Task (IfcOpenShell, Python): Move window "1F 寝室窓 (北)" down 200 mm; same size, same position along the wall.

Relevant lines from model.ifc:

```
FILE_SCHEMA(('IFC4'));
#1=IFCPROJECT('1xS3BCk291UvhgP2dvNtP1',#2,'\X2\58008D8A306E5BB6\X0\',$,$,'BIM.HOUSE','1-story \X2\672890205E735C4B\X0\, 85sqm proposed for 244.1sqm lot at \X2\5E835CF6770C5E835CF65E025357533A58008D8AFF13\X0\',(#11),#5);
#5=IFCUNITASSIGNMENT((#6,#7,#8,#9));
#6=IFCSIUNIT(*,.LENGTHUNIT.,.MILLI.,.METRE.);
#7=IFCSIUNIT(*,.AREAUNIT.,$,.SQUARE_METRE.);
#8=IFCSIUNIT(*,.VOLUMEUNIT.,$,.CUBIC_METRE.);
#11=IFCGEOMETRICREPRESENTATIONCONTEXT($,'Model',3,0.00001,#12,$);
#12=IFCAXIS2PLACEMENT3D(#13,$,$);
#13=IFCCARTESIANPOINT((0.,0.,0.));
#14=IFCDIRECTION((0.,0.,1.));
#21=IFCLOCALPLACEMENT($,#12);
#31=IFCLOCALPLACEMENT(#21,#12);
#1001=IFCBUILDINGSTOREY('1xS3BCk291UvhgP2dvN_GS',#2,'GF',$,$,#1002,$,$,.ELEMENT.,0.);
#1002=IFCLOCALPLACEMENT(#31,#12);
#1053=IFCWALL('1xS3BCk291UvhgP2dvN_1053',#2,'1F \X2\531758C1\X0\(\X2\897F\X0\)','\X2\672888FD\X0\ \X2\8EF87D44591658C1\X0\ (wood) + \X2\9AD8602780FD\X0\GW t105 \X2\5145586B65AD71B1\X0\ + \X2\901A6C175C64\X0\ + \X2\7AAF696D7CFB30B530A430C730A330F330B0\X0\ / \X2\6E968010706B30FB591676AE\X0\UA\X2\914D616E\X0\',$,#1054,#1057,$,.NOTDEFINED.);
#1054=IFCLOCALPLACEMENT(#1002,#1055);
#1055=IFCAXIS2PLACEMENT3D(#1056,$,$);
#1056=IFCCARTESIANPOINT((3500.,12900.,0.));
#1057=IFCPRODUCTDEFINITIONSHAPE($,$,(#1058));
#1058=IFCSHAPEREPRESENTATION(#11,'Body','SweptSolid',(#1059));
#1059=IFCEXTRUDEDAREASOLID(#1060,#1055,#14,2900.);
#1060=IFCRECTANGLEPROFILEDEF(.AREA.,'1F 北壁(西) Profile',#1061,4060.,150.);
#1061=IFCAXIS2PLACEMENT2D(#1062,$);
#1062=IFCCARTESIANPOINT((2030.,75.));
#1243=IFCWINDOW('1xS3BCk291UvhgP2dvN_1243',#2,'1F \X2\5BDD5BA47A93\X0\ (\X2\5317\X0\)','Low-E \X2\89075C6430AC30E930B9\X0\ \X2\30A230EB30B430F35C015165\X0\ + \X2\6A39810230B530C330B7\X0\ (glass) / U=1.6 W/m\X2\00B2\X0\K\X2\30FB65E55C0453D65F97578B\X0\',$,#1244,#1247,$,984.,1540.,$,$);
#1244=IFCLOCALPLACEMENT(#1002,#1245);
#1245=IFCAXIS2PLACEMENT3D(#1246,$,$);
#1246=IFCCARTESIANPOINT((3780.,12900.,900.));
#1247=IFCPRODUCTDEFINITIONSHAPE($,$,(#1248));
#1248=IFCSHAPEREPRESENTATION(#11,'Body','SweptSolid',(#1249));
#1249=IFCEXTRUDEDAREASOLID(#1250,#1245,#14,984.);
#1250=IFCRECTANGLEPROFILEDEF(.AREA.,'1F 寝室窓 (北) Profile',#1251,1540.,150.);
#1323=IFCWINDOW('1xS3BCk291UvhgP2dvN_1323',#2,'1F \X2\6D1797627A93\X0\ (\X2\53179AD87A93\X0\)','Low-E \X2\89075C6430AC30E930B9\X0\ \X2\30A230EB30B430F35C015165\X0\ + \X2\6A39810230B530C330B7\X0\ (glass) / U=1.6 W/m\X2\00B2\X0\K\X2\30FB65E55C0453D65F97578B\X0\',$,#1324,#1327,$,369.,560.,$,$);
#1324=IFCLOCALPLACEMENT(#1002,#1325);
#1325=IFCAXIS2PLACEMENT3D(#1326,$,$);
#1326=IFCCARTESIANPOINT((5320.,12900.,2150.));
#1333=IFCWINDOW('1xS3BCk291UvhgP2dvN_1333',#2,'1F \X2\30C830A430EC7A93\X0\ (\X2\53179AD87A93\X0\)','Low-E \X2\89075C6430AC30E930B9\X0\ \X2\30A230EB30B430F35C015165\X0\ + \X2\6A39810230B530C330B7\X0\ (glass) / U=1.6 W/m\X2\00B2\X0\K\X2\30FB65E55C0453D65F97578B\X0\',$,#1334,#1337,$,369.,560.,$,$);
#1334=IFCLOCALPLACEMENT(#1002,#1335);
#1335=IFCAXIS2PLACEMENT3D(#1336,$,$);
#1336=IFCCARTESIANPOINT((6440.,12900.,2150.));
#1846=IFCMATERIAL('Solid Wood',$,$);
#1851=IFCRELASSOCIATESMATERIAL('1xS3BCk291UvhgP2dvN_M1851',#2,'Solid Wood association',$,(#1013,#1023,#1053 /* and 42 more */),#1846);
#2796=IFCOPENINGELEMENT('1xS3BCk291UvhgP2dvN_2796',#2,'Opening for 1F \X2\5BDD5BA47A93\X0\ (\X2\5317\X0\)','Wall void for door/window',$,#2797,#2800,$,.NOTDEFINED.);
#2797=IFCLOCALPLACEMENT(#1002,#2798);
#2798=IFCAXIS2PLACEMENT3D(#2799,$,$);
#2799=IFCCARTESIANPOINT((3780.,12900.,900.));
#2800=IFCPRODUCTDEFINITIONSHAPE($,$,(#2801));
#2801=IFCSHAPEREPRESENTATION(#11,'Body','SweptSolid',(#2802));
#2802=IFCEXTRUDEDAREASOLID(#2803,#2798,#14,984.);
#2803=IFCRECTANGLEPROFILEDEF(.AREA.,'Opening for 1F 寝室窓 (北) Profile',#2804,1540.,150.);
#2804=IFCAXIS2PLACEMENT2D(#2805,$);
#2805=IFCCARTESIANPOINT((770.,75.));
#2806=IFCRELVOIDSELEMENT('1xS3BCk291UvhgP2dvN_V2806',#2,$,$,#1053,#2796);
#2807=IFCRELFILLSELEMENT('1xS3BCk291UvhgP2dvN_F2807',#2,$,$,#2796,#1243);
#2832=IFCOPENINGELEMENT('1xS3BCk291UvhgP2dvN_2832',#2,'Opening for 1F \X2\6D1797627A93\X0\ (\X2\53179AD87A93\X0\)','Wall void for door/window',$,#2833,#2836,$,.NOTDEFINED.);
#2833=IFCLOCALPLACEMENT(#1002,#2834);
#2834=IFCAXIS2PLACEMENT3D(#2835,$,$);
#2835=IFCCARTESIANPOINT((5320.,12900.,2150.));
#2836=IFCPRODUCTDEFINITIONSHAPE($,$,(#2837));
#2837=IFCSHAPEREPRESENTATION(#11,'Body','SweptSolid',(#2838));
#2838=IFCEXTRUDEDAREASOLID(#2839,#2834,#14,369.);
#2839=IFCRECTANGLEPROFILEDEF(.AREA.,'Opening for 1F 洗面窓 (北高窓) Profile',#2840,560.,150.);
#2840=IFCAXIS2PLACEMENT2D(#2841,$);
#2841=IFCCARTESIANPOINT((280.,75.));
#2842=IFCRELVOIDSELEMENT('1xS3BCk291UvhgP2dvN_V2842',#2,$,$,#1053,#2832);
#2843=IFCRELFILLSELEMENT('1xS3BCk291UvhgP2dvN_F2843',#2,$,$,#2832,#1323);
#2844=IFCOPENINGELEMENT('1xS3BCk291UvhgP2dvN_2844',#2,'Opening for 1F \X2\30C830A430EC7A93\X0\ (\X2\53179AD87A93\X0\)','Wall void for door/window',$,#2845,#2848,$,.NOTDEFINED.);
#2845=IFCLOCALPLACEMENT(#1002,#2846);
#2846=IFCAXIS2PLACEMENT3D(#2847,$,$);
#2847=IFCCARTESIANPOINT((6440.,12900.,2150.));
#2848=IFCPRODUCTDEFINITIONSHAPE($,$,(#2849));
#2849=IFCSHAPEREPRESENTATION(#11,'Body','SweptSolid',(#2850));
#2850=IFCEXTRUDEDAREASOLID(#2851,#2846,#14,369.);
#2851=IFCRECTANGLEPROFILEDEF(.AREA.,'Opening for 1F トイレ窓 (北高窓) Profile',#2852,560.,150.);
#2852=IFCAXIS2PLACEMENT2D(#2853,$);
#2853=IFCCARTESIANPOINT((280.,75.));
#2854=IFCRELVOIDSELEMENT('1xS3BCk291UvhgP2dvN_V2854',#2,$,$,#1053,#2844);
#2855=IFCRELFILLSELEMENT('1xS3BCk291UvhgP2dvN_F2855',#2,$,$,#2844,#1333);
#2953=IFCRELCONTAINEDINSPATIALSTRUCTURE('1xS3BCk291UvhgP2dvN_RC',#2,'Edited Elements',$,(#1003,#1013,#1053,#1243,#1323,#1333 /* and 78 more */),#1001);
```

```python
import numpy as np
import ifcopenshell
import ifcopenshell.api.geometry
import ifcopenshell.util.placement
import ifcopenshell.util.unit

model = ifcopenshell.open("model.ifc")
unit_scale = ifcopenshell.util.unit.calculate_unit_scale(model)

window = model.by_id(1243)
opening = window.FillsVoids[0].RelatingOpeningElement
dz = -0.2 / unit_scale

shift = np.array([0.0, 0.0, dz])
# The window is not placed relative to its opening, so move both.
for product in (opening, window):
    matrix = ifcopenshell.util.placement.get_local_placement(product.ObjectPlacement)
    matrix[:3, 3] += shift
    ifcopenshell.api.geometry.edit_object_placement(model, product=product, matrix=matrix, is_si=False)

print(f"moved by {dz * unit_scale:+.3f} m")

model.write("model_rev.ifc")
```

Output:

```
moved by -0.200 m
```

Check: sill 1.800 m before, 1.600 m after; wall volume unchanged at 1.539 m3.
